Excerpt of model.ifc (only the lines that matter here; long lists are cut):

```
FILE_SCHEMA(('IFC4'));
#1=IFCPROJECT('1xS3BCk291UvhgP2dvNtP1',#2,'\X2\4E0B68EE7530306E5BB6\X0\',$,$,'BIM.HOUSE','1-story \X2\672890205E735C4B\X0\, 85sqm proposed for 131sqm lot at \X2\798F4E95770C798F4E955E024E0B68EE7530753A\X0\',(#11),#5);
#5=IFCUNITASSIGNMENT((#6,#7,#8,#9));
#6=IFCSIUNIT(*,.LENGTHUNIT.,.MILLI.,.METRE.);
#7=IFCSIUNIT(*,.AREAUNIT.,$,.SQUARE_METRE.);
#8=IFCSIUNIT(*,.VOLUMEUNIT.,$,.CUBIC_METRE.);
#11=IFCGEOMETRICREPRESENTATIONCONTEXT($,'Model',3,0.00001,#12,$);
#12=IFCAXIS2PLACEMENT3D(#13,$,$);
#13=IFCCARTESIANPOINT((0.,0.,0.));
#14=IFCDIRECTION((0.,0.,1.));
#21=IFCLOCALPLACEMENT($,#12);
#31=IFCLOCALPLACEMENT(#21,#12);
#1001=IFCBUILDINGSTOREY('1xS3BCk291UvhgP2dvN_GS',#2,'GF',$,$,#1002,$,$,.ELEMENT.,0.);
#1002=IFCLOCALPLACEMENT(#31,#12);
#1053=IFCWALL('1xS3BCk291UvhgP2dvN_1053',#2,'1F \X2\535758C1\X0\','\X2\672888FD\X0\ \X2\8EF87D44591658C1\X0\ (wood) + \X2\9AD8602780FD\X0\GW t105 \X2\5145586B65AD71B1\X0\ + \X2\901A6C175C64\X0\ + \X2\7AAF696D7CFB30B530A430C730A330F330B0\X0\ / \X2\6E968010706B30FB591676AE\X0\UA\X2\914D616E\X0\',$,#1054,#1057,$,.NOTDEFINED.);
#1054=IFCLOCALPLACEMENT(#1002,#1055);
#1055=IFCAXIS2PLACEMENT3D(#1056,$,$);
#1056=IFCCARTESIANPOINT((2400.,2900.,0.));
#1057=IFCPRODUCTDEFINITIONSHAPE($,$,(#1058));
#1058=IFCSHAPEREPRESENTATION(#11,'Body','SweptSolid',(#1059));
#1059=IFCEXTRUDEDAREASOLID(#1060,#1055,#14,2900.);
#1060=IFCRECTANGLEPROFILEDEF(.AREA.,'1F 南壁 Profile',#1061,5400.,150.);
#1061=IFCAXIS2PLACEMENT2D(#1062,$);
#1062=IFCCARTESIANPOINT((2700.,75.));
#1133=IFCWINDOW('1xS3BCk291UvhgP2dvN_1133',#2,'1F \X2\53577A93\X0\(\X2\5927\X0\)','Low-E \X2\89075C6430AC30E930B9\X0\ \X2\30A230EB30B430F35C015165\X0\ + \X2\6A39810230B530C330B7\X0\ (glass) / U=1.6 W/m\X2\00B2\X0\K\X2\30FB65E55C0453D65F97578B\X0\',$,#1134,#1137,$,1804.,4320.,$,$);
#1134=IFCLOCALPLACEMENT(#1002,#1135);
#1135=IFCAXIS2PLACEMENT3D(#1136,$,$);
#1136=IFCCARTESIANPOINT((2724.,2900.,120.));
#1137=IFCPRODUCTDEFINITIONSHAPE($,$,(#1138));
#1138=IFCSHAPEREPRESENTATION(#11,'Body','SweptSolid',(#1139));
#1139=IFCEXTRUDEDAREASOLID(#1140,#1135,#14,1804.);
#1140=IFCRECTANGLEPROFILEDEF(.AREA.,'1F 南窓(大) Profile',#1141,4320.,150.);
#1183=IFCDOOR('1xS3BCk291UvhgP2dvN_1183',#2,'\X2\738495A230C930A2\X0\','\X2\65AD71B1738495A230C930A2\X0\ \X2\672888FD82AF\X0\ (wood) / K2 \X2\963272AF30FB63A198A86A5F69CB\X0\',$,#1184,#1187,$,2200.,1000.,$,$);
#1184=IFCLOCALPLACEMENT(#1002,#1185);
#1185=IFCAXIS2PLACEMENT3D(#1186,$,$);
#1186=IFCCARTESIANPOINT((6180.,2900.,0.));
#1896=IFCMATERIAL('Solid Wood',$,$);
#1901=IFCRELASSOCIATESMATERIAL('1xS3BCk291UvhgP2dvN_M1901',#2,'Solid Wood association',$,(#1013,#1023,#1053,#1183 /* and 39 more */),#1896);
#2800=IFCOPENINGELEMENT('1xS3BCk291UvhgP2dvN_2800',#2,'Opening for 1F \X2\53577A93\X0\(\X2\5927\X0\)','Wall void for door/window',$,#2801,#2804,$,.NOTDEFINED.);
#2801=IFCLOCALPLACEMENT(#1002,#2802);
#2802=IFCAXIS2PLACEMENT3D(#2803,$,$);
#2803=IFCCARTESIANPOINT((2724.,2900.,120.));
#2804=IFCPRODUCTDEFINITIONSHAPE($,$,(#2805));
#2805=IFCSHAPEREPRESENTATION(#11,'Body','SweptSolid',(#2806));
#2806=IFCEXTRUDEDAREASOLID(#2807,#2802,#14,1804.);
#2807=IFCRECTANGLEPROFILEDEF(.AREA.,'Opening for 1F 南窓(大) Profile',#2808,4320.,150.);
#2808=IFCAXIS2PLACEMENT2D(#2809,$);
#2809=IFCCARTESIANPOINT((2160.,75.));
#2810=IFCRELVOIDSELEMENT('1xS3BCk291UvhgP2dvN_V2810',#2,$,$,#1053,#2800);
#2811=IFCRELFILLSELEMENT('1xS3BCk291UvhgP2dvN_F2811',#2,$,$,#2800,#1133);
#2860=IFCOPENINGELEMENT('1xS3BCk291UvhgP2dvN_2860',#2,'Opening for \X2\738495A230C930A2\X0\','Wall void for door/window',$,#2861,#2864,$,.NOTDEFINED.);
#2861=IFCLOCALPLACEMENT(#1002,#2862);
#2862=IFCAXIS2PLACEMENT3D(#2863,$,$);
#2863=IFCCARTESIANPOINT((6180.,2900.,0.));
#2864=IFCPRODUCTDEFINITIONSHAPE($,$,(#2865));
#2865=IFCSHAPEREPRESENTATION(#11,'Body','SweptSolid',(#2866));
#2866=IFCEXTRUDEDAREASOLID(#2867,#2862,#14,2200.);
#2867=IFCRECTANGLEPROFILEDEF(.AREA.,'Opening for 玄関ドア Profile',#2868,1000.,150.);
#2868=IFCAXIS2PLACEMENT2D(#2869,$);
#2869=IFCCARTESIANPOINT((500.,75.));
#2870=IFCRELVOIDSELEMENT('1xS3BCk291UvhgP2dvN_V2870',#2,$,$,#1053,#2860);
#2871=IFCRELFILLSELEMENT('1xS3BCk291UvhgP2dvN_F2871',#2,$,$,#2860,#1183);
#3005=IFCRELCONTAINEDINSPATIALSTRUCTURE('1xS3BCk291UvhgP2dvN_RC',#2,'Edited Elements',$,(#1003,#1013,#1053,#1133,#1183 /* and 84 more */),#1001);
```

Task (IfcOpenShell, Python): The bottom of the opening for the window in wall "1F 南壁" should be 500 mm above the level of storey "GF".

```python
import numpy as np
import ifcopenshell
import ifcopenshell.api.geometry
import ifcopenshell.geom
import ifcopenshell.util.element
import ifcopenshell.util.placement
import ifcopenshell.util.shape
import ifcopenshell.util.unit

model = ifcopenshell.open("model.ifc")
unit_scale = ifcopenshell.util.unit.calculate_unit_scale(model)

window = model.by_guid("1xS3BCk291UvhgP2dvN_1133")
opening = window.FillsVoids[0].RelatingOpeningElement
storey = ifcopenshell.util.element.get_container(window, ifc_class="IfcBuildingStorey")
level = ifcopenshell.util.placement.get_local_placement(storey.ObjectPlacement)[2, 3]

# The opening's origin need not be at the sill, so measure its lowest point.
shape = ifcopenshell.geom.create_shape(ifcopenshell.geom.settings(), opening)
bottom = ifcopenshell.util.shape.get_shape_bottom_elevation(shape, shape.geometry) / unit_scale
dz = level + 0.5 / unit_scale - bottom

shift = np.array([0.0, 0.0, dz])
# The window is not placed relative to its opening, so move both.
for product in (opening, window):
    matrix = ifcopenshell.util.placement.get_local_placement(product.ObjectPlacement)
    matrix[:3, 3] += shift
    ifcopenshell.api.geometry.edit_object_placement(model, product=product, matrix=matrix, is_si=False)

print(f"moved by {dz * unit_scale:+.3f} m")

model.write("model_updated.ifc")
```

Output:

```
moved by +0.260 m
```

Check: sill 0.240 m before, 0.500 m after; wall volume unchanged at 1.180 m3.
